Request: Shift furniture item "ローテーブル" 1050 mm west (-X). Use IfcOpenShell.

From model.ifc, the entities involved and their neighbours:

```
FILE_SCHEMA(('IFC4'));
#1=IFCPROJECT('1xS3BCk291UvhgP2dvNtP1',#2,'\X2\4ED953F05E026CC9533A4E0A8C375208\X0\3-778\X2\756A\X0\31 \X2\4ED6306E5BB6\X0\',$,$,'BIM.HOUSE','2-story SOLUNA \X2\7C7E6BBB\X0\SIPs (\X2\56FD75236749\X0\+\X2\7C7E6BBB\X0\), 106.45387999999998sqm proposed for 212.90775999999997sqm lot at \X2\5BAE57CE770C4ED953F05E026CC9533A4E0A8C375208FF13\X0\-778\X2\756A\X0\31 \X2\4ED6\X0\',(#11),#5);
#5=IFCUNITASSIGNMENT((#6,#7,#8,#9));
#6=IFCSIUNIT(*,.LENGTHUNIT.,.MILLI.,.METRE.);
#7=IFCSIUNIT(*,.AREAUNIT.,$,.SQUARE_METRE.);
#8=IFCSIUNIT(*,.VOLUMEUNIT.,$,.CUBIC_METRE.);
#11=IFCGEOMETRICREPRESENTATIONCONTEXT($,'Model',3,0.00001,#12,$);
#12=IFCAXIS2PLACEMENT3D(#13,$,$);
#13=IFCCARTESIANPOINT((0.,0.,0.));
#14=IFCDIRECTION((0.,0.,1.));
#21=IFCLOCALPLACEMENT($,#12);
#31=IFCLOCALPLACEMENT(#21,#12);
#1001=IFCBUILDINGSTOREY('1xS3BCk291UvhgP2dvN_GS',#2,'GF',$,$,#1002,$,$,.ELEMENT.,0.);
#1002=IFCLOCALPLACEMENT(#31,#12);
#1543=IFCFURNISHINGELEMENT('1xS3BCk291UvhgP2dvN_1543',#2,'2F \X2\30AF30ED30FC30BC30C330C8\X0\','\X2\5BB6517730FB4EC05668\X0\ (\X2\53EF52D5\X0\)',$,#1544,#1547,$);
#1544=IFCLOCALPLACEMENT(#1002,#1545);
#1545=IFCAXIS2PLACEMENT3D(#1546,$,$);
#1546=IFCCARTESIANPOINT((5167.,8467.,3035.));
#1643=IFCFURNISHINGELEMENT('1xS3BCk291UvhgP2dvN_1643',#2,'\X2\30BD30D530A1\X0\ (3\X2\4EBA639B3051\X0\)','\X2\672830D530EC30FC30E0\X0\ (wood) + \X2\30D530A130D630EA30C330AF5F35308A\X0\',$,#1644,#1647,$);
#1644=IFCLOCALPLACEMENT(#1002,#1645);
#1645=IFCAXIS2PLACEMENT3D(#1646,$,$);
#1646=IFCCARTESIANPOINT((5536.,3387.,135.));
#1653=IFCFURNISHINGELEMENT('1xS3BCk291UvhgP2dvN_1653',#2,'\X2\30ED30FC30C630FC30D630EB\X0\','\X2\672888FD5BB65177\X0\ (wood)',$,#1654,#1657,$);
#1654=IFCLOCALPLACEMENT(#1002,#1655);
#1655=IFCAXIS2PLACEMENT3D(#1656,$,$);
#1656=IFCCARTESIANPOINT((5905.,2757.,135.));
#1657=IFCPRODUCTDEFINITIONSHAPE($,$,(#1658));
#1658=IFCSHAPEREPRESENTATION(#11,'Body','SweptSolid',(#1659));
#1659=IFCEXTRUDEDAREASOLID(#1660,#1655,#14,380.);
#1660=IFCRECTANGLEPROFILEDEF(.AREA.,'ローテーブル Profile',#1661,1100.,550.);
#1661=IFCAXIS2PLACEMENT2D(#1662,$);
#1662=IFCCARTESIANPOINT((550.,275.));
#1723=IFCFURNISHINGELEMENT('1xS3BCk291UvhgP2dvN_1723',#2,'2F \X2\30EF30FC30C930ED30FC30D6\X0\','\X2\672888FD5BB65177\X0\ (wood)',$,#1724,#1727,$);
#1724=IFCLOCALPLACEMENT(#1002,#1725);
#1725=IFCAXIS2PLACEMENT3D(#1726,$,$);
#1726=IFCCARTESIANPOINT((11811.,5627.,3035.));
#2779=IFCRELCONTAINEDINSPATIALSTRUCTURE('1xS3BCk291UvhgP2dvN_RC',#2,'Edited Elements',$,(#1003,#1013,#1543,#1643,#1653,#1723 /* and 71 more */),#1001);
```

```python
import ifcopenshell
import ifcopenshell.api.geometry
import ifcopenshell.util.placement

model = ifcopenshell.open("model.ifc")

item = model.by_id(1653)
matrix = ifcopenshell.util.placement.get_local_placement(item.ObjectPlacement)
matrix[0, 3] -= 1050.0
ifcopenshell.api.geometry.edit_object_placement(model, product=item, matrix=matrix, is_si=False)

print(ifcopenshell.util.placement.get_local_placement(item.ObjectPlacement).round(3) + 0.0)

model.write("model_edited.ifc")
```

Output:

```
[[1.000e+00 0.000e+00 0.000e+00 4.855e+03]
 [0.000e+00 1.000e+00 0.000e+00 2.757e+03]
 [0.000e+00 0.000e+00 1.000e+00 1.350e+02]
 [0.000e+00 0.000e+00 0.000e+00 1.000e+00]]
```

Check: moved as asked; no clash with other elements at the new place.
